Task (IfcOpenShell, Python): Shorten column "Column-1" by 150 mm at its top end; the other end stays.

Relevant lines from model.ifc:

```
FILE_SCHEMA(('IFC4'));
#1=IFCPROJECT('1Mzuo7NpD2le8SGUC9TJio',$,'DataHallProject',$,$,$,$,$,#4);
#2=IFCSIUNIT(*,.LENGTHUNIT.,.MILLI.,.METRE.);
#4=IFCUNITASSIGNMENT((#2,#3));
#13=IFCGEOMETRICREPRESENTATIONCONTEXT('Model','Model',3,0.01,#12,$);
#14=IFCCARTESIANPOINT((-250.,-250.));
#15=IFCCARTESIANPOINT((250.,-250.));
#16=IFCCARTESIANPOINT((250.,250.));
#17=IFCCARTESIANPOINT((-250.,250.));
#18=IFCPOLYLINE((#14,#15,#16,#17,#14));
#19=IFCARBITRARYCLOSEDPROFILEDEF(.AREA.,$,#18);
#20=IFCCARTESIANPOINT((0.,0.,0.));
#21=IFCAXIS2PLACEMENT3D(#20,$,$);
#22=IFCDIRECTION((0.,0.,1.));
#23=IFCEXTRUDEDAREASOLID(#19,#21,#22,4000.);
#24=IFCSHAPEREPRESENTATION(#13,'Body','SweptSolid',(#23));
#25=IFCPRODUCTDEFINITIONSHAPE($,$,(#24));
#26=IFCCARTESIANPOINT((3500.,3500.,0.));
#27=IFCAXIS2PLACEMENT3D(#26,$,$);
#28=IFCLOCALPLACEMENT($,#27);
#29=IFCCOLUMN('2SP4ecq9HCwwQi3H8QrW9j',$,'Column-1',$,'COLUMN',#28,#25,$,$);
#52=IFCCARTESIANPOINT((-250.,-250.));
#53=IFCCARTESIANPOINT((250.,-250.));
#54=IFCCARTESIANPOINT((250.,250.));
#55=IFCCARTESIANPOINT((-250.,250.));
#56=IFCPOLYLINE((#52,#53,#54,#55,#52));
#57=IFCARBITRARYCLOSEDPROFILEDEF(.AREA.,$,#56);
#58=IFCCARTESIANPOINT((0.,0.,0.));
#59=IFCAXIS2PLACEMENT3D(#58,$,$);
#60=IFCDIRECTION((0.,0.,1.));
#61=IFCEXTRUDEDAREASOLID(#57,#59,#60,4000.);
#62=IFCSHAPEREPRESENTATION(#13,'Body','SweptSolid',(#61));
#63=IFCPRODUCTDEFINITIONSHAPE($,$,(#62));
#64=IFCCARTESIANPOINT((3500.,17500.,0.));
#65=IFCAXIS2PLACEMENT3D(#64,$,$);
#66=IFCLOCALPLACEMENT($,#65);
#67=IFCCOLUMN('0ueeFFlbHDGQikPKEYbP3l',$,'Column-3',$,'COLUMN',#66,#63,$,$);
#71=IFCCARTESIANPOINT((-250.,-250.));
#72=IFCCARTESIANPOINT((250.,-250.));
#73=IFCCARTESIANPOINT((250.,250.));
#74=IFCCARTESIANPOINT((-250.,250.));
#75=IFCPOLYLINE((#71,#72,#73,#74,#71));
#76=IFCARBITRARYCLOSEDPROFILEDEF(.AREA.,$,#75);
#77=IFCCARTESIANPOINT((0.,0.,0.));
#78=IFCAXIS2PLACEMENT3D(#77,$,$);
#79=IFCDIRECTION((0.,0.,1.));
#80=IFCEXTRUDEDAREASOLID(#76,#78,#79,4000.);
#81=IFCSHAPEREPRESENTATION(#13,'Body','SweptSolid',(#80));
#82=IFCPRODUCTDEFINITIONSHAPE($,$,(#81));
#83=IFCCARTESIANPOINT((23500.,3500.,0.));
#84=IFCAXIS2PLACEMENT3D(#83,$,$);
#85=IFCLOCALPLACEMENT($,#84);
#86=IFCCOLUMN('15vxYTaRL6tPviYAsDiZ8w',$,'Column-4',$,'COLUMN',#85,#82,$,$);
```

```python
import ifcopenshell
import ifcopenshell.util.unit

model = ifcopenshell.open("model.ifc")
unit_scale = ifcopenshell.util.unit.calculate_unit_scale(model)

member = model.by_guid("2SP4ecq9HCwwQi3H8QrW9j")
change = -0.15 / unit_scale

# The extrusion runs towards the end named, so only its depth changes.
body = next(r for r in member.Representation.Representations if r.RepresentationIdentifier == "Body")
solid = body.Items[0]
old_length = solid.Depth
solid.Depth += change

print(f"length {old_length:g} -> {solid.Depth:g}")

model.write("model-out.ifc")
```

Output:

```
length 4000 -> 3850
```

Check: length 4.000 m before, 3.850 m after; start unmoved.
